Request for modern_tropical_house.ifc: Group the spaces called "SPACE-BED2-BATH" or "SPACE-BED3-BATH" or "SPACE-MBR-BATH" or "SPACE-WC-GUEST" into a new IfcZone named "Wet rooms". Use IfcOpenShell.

First a look at what the model holds.

```python
import ifcopenshell

model = ifcopenshell.open("modern_tropical_house.ifc")
print(model.schema)
seen = {}
for space in model.by_type("IfcSpace"):
    seen[space.Name] = seen.get(space.Name, 0) + 1
for name, count in sorted(seen.items(), key=str):
    print(count, "x", name)
print("zones:", [z.Name for z in model.by_type("IfcZone")][:20])
```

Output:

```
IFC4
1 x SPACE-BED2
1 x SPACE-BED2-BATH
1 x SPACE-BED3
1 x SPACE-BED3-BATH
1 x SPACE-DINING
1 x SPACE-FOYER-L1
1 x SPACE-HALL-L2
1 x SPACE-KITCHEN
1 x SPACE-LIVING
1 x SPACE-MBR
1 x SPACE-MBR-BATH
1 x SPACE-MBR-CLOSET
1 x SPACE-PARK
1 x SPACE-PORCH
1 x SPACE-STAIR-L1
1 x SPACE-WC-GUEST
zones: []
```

```python
import ifcopenshell
import ifcopenshell.api.group
import ifcopenshell.api.root

model = ifcopenshell.open("modern_tropical_house.ifc")

names = {"SPACE-BED2-BATH", "SPACE-BED3-BATH", "SPACE-MBR-BATH", "SPACE-WC-GUEST"}
spaces = [s for s in model.by_type("IfcSpace") if s.Name in names]

zone = ifcopenshell.api.root.create_entity(model, ifc_class="IfcZone", name="Wet rooms")
ifcopenshell.api.group.assign_group(model, products=spaces, group=zone)
print(len(spaces), "spaces in", zone.Name)

model.write("modern_tropical_house_rev.ifc")
```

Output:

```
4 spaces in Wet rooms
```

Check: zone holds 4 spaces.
